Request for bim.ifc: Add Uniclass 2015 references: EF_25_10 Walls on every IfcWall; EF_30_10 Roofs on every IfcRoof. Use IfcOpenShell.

First a look at what the model holds.

```python
import ifcopenshell

model = ifcopenshell.open("bim.ifc")
print(model.schema)
print("classifications:", [c.Name for c in model.by_type("IfcClassification")])
for ifc_class in ("IfcDoor", "IfcRoof", "IfcStair", "IfcWall", "IfcWindow"):
    print(ifc_class, len(model.by_type(ifc_class)))
```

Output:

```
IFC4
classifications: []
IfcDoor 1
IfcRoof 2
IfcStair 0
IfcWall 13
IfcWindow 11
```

```python
import ifcopenshell
import ifcopenshell.api.classification

model = ifcopenshell.open("bim.ifc")

system = ifcopenshell.api.classification.add_classification(model, classification="Uniclass 2015")

codes = {
    "IfcWall": ("EF_25_10", "Walls"),
    "IfcRoof": ("EF_30_10", "Roofs"),
}
for ifc_class, (code, name) in codes.items():
    products = model.by_type(ifc_class)
    ifcopenshell.api.classification.add_reference(
        model, products=products, classification=system, identification=code, name=name
    )
    print(code, len(products))

model.write("bim_v2.ifc")
```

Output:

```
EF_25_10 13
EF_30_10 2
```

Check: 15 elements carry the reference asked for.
